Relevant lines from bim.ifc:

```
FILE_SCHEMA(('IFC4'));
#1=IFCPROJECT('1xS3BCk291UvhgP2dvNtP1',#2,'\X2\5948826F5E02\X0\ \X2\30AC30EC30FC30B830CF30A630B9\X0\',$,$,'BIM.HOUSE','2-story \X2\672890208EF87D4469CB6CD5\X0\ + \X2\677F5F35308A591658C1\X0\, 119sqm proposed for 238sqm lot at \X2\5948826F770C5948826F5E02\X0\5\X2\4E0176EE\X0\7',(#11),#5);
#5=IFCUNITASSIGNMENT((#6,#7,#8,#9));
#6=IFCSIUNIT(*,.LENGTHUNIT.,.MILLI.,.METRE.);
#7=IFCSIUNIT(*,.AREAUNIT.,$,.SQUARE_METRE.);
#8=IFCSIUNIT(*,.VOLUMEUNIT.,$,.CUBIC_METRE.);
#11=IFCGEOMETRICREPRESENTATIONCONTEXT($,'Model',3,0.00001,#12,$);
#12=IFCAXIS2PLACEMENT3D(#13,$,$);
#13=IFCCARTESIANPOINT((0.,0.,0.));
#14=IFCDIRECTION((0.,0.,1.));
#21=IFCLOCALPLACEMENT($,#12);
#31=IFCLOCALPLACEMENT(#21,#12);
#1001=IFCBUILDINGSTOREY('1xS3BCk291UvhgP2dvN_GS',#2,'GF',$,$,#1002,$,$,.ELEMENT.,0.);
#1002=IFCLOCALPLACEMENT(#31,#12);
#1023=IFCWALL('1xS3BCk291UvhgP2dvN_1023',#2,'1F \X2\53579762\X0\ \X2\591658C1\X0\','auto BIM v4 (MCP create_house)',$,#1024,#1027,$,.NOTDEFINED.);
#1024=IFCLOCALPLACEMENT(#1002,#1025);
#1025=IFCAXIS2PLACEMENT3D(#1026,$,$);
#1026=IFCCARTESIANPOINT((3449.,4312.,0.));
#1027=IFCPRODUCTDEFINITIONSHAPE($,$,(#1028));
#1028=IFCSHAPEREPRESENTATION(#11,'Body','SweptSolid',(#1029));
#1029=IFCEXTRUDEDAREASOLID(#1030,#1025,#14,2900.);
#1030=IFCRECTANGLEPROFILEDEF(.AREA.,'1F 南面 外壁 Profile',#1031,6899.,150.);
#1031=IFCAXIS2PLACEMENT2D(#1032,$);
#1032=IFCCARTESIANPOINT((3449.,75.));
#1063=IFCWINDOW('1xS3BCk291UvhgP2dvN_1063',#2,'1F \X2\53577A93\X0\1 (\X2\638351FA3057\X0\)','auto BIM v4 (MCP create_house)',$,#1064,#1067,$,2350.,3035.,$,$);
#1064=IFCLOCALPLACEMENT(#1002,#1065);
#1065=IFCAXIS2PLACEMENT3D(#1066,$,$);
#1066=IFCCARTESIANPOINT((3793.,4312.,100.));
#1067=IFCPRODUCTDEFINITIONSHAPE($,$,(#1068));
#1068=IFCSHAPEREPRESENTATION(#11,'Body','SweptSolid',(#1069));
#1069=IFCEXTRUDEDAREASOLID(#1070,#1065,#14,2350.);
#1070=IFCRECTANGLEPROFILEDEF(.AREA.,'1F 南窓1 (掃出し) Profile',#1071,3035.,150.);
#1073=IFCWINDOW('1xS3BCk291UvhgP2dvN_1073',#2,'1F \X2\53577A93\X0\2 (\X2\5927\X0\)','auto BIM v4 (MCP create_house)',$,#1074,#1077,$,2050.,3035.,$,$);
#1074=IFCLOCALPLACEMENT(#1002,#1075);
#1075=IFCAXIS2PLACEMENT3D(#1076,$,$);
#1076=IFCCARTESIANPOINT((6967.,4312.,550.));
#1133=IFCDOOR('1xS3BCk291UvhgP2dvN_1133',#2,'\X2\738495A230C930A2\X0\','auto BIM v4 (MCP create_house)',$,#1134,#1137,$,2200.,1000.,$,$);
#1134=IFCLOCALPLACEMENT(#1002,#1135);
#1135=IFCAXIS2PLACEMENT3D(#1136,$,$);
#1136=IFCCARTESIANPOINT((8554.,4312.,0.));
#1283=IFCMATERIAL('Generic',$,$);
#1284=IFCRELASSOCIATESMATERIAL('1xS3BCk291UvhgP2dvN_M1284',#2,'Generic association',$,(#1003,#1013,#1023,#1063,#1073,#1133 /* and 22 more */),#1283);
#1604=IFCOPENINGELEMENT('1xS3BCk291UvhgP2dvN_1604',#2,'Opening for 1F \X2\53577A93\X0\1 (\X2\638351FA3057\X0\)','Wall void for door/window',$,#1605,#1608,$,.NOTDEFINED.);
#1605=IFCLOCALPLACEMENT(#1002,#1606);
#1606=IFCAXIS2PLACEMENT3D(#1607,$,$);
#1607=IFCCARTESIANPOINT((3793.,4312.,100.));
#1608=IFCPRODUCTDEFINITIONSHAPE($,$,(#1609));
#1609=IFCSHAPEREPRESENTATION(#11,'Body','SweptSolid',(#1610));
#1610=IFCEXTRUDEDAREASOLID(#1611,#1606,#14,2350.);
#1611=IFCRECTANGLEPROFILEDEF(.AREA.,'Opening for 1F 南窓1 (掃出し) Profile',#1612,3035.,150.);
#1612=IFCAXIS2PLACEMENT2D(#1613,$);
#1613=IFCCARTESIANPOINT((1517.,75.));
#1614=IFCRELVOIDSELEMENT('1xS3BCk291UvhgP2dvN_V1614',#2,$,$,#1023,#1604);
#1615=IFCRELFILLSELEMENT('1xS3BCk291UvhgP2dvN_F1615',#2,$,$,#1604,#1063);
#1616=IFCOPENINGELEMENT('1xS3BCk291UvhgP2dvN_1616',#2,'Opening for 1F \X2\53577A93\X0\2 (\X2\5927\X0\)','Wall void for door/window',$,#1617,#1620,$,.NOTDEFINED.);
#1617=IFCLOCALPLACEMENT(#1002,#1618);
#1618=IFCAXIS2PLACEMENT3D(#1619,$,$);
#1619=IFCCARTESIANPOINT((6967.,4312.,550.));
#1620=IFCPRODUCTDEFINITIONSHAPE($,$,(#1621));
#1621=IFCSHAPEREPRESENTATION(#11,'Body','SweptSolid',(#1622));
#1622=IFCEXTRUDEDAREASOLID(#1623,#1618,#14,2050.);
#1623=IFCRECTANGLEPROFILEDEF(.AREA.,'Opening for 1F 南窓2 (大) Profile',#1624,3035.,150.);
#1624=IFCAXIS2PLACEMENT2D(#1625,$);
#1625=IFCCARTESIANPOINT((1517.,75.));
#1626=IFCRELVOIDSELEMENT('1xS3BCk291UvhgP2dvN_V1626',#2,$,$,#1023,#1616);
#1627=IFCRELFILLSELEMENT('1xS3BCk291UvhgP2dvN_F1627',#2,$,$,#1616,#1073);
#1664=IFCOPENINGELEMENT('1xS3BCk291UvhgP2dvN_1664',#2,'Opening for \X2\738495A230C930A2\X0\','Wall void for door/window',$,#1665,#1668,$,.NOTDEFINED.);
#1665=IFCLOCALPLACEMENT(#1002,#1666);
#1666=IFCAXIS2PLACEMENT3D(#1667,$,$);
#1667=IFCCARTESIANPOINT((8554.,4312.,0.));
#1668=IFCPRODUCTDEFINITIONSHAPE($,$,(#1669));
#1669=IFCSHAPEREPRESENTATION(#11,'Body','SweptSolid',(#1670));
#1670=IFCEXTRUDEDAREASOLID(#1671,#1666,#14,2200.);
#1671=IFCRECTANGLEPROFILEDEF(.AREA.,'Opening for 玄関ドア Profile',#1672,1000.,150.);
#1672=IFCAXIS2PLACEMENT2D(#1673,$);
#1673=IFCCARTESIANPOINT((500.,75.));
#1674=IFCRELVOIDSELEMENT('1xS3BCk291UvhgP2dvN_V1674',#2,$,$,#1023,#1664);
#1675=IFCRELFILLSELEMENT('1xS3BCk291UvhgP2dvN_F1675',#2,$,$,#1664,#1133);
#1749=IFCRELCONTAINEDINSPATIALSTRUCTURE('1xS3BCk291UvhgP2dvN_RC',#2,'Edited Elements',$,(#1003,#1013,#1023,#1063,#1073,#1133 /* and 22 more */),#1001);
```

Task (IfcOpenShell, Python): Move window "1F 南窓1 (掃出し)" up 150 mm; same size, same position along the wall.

```python
import numpy as np
import ifcopenshell
import ifcopenshell.api.geometry
import ifcopenshell.util.placement
import ifcopenshell.util.unit

model = ifcopenshell.open("bim.ifc")
unit_scale = ifcopenshell.util.unit.calculate_unit_scale(model)

window = model.by_guid("1xS3BCk291UvhgP2dvN_1063")
opening = window.FillsVoids[0].RelatingOpeningElement
dz = 150.0

shift = np.array([0.0, 0.0, dz])
# The window is not placed relative to its opening, so move both.
for product in (opening, window):
    matrix = ifcopenshell.util.placement.get_local_placement(product.ObjectPlacement)
    matrix[:3, 3] += shift
    ifcopenshell.api.geometry.edit_object_placement(model, product=product, matrix=matrix, is_si=False)

print(f"moved by {dz * unit_scale:+.3f} m")

model.write("bim_edited.ifc")
```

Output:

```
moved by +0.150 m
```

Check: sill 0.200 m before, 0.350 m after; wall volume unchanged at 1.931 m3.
